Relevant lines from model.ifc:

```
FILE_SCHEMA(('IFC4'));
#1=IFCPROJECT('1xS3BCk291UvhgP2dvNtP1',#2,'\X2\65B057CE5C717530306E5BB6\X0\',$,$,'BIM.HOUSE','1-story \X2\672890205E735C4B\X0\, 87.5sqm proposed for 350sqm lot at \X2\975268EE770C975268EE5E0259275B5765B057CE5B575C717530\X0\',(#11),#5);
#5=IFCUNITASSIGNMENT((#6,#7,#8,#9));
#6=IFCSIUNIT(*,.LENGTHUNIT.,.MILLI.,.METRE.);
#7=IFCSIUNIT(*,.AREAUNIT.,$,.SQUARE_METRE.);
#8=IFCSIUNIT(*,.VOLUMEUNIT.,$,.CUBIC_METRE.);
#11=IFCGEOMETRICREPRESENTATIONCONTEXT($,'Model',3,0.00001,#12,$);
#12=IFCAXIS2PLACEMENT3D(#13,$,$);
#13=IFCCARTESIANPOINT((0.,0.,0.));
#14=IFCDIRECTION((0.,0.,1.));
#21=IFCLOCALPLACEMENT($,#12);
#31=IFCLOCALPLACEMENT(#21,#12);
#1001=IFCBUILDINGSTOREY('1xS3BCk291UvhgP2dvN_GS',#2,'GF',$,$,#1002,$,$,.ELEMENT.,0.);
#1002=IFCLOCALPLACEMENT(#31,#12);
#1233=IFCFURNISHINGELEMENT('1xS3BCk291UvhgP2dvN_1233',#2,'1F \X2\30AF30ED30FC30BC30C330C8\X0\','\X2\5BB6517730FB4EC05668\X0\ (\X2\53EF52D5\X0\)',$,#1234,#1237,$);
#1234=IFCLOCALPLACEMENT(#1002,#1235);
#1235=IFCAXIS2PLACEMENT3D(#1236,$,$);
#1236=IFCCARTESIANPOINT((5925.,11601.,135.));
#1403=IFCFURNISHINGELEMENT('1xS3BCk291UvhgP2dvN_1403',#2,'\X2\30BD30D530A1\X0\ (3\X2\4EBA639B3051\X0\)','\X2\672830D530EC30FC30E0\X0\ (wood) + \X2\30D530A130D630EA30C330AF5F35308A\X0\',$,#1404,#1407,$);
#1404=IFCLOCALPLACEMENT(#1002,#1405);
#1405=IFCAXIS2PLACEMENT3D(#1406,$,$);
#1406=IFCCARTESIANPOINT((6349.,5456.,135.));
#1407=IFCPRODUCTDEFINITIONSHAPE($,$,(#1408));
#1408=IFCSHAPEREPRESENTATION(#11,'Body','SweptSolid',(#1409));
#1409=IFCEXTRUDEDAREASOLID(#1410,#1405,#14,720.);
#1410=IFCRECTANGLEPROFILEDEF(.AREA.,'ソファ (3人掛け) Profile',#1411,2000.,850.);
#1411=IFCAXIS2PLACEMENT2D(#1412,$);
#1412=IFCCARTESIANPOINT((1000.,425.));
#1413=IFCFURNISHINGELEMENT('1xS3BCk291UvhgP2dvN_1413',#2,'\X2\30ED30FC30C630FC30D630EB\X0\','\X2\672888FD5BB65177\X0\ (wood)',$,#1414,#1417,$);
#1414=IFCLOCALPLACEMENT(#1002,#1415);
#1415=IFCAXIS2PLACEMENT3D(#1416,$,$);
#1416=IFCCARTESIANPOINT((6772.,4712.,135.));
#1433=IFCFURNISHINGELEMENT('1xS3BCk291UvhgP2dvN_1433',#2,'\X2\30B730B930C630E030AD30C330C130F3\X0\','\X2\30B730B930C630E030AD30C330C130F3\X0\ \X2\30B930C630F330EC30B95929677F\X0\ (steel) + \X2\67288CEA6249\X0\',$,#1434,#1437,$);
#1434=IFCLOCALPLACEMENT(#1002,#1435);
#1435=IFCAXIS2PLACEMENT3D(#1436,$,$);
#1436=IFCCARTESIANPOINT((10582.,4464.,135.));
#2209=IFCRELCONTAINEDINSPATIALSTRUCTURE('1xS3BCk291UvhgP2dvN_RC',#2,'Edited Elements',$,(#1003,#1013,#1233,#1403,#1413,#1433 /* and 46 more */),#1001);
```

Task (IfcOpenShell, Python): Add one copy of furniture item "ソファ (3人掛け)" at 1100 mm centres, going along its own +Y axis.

```python
import ifcopenshell
import ifcopenshell.api.geometry
import ifcopenshell.api.root
import ifcopenshell.util.element
import ifcopenshell.util.placement
import ifcopenshell.util.unit

model = ifcopenshell.open("model.ifc")
unit_scale = ifcopenshell.util.unit.calculate_unit_scale(model)


def reuse_history(source, copy):
    """copy_class also copies each property set's owner history, people and application; keep the originals."""
    for rel in copy.IsDefinedBy:
        if rel.is_a("IfcRelDefinesByProperties") and (history := rel.RelatingPropertyDefinition.OwnerHistory):
            rel.RelatingPropertyDefinition.OwnerHistory = source.OwnerHistory
            ifcopenshell.util.element.remove_deep2(model, history)


source = model.by_id(1403)
base = ifcopenshell.util.placement.get_local_placement(source.ObjectPlacement)
step = base[:3, 1] * 1.1 / unit_scale

for i in range(1, 2):
    copy = ifcopenshell.api.root.copy_class(model, product=source)
    copy.Representation = ifcopenshell.util.element.copy_deep(
        model, source.Representation, exclude=["IfcGeometricRepresentationContext", "IfcRepresentationMap"]
    )
    reuse_history(source, copy)
    matrix = base.copy()
    matrix[:3, 3] += i * step
    print("added at", matrix[:3, 3].round(3) + 0.0)
    ifcopenshell.api.geometry.edit_object_placement(model, product=copy, matrix=matrix, is_si=False)

model.write("model_edited.ifc")
```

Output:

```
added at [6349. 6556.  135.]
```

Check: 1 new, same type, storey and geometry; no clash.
